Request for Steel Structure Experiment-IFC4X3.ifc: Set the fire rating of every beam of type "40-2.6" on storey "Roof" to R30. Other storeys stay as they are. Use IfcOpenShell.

First a look at what the model holds.

```python
import ifcopenshell
import ifcopenshell.util.element

model = ifcopenshell.open("Steel Structure Experiment-IFC4X3.ifc")
print(model.schema)
storey = next(s for s in model.by_type("IfcBuildingStorey") if s.Name == "Roof")
beams = [e for e in ifcopenshell.util.element.get_decomposition(storey) if e.is_a("IfcBeam")]
seen = {}
for e in beams:
    element_type = ifcopenshell.util.element.get_type(e)
    key = (element_type.Name if element_type != e and element_type else None, ifcopenshell.util.element.get_pset(e, "Pset_BeamCommon", "FireRating"))
    seen[key] = seen.get(key, 0) + 1
for (name, value), count in sorted(seen.items(), key=str):
    print(count, "x", name, "|", value)
```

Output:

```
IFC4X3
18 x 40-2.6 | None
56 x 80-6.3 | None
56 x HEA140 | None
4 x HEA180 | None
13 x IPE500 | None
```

```python
import ifcopenshell
import ifcopenshell.api.pset
import ifcopenshell.util.element

model = ifcopenshell.open("Steel Structure Experiment-IFC4X3.ifc")

storey = next(s for s in model.by_type("IfcBuildingStorey") if s.Name == "Roof")
beams = [e for e in ifcopenshell.util.element.get_decomposition(storey) if e.is_a("IfcBeam")]

count = 0
for e in beams:
    element_type = ifcopenshell.util.element.get_type(e)
    if element_type in (None, e) or element_type.Name != "40-2.6":
        continue
    # add_pset returns the element's existing set when there is one.
    pset = ifcopenshell.api.pset.add_pset(model, product=e, name="Pset_BeamCommon")
    ifcopenshell.api.pset.edit_pset(model, pset=pset, properties={"FireRating": "R30"})
    count += 1

print(count, "beams updated")

model.write("Steel Structure Experiment-IFC4X3_v2.ifc")
```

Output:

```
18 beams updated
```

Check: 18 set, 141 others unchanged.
